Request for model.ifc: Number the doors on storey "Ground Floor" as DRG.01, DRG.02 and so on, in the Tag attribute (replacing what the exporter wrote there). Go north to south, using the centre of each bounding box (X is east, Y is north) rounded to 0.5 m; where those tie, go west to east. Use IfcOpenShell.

First a look at what the model holds.

```python
import ifcopenshell
import ifcopenshell.util.element
import ifcopenshell.util.placement

model = ifcopenshell.open("model.ifc")
print(model.schema)
storey = next(s for s in model.by_type("IfcBuildingStorey") if s.Name == "Ground Floor")
doors = [e for e in ifcopenshell.util.element.get_decomposition(storey) if e.is_a("IfcDoor")]
for e in sorted(doors, key=lambda e: e.id()):
    origin = ifcopenshell.util.placement.get_local_placement(e.ObjectPlacement)[:3, 3]
    print(e.id(), e.Tag, e.Name, origin.round(2) + 0.0, sep=" | ")
```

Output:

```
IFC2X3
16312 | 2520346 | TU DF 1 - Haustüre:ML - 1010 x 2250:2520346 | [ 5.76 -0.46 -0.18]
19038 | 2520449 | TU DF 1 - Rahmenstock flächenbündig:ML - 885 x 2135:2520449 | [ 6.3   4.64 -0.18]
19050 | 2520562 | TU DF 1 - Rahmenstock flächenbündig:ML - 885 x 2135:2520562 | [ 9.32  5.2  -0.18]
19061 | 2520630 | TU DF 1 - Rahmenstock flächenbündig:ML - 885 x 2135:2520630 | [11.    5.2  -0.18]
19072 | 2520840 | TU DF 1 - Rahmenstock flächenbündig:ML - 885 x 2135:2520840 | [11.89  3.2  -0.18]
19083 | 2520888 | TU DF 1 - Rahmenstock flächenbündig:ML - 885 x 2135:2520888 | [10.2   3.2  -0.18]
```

```python
import ifcopenshell
import ifcopenshell.geom
import ifcopenshell.util.element
import ifcopenshell.util.shape

model = ifcopenshell.open("model.ifc")
settings = ifcopenshell.geom.settings()
settings.set("use-world-coords", True)


def centre(element):
    shape = ifcopenshell.geom.create_shape(settings, element)
    return ifcopenshell.util.shape.get_bbox_centroid(shape.geometry)


storey = next(s for s in model.by_type("IfcBuildingStorey") if s.Name == "Ground Floor")
doors = [e for e in ifcopenshell.util.element.get_decomposition(storey) if e.is_a("IfcDoor")]

# Insertion points can sit at a corner or the storey origin, so sort by the geometry (in metres).
centres = {e: centre(e) for e in doors}
doors.sort(key=lambda e: (-round(centres[e][1] / 0.5), centres[e][0]))

for i, e in enumerate(doors, start=1):
    number = f"DRG.{i:02d}"
    e.Tag = number
    print(e.id(), number)

model.write("model_updated.ifc")
```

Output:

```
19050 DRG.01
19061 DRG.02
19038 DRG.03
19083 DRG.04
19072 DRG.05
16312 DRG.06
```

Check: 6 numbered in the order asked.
